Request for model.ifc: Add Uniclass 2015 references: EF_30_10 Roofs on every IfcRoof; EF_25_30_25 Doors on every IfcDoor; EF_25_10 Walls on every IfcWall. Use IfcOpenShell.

First a look at what the model holds.

```python
import ifcopenshell

model = ifcopenshell.open("model.ifc")
print(model.schema)
print("classifications:", [c.Name for c in model.by_type("IfcClassification")])
for ifc_class in ("IfcDoor", "IfcRoof", "IfcStair", "IfcWall", "IfcWindow"):
    print(ifc_class, len(model.by_type(ifc_class)))
```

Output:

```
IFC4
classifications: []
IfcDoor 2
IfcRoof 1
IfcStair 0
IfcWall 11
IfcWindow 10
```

```python
import ifcopenshell
import ifcopenshell.api.classification

model = ifcopenshell.open("model.ifc")

system = ifcopenshell.api.classification.add_classification(model, classification="Uniclass 2015")

codes = {
    "IfcRoof": ("EF_30_10", "Roofs"),
    "IfcDoor": ("EF_25_30_25", "Doors"),
    "IfcWall": ("EF_25_10", "Walls"),
}
for ifc_class, (code, name) in codes.items():
    products = model.by_type(ifc_class)
    ifcopenshell.api.classification.add_reference(
        model, products=products, classification=system, identification=code, name=name
    )
    print(code, len(products))

model.write("model_rev.ifc")
```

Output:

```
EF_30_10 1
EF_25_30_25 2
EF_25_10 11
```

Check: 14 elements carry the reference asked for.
